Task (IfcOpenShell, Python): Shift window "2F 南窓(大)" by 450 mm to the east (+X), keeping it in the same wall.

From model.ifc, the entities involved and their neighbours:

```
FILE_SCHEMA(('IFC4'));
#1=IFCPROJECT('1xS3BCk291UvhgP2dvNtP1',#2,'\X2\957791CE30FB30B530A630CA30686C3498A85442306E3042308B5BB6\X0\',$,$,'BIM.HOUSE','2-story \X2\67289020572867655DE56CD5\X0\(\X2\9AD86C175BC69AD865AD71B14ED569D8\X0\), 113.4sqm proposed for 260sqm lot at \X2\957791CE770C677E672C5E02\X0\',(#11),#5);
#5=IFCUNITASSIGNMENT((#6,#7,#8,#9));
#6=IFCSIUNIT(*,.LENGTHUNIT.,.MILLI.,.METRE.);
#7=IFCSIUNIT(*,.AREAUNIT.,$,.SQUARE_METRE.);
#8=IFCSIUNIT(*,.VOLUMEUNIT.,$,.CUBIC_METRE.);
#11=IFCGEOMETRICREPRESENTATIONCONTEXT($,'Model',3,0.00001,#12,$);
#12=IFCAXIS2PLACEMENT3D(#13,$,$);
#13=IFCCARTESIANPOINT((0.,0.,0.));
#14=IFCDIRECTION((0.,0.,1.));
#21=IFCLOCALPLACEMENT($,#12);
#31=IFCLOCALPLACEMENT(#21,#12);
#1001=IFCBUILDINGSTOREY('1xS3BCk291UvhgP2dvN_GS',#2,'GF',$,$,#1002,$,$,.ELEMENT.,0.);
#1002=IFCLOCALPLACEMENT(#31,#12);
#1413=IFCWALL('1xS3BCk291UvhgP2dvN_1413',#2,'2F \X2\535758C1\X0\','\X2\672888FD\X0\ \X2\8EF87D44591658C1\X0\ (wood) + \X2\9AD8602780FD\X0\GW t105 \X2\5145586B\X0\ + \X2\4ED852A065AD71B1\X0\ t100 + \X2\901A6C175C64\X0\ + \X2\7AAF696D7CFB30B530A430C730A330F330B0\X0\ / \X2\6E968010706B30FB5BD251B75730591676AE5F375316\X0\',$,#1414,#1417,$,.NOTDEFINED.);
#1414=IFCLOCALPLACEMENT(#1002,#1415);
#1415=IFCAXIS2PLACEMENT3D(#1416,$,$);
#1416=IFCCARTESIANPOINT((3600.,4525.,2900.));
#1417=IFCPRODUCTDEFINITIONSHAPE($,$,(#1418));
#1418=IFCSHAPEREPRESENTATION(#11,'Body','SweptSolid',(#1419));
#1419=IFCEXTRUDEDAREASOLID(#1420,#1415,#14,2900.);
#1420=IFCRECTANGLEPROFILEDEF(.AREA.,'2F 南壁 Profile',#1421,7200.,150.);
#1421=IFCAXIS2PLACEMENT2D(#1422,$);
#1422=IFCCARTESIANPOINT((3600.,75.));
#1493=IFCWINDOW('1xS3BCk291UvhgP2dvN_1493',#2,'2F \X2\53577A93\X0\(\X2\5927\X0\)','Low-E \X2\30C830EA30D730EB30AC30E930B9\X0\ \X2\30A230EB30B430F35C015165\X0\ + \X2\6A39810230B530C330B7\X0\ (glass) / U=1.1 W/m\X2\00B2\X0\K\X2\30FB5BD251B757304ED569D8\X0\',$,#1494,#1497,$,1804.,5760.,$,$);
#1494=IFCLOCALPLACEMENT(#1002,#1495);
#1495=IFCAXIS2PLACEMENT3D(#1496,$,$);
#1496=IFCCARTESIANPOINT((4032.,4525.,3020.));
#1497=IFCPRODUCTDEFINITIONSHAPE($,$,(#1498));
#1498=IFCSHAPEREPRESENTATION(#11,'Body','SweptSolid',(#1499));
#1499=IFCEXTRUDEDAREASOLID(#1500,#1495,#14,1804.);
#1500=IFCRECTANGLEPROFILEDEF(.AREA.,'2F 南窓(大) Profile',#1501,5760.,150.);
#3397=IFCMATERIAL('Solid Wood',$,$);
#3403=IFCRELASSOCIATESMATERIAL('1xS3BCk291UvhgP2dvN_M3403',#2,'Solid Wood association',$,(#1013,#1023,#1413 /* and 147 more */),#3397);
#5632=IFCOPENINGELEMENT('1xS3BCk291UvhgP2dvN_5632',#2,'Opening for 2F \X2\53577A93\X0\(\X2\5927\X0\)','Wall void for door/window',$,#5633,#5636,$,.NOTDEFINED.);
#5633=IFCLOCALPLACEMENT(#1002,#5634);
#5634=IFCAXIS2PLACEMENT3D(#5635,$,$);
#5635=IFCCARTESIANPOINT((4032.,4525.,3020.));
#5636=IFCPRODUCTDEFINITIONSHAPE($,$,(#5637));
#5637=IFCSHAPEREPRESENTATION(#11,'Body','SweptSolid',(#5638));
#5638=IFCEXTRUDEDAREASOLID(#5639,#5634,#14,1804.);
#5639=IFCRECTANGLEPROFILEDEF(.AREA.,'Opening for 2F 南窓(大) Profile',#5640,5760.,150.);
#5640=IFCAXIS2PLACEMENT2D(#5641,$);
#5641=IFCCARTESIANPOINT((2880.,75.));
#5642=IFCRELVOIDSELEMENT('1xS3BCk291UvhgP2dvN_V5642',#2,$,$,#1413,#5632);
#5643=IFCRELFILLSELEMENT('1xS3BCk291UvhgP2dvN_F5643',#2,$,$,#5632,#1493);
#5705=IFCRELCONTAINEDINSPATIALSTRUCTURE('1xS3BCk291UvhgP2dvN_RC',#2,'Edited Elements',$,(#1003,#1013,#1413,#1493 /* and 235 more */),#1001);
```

```python
import ifcopenshell
import ifcopenshell.api.geometry
import ifcopenshell.util.placement
import ifcopenshell.util.unit

model = ifcopenshell.open("model.ifc")
unit_scale = ifcopenshell.util.unit.calculate_unit_scale(model)

window = model.by_guid("1xS3BCk291UvhgP2dvN_1493")
opening = window.FillsVoids[0].RelatingOpeningElement
wall = opening.VoidsElements[0].RelatingBuildingElement

wall_matrix = ifcopenshell.util.placement.get_local_placement(wall.ObjectPlacement)
shift = wall_matrix[:3, 0] * 0.45 / unit_scale
before = ifcopenshell.util.placement.get_local_placement(window.ObjectPlacement)[:3, 3].copy()

# The window is not placed relative to its opening, so move both.
for product in (opening, window):
    matrix = ifcopenshell.util.placement.get_local_placement(product.ObjectPlacement)
    matrix[:3, 3] += shift
    ifcopenshell.api.geometry.edit_object_placement(model, product=product, matrix=matrix, is_si=False)

after = ifcopenshell.util.placement.get_local_placement(window.ObjectPlacement)[:3, 3]
print("window moved by", (after - before).round(3) + 0.0)

model.write("model_edited.ifc")
```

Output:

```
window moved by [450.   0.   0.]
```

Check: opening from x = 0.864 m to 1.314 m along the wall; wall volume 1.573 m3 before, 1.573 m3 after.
